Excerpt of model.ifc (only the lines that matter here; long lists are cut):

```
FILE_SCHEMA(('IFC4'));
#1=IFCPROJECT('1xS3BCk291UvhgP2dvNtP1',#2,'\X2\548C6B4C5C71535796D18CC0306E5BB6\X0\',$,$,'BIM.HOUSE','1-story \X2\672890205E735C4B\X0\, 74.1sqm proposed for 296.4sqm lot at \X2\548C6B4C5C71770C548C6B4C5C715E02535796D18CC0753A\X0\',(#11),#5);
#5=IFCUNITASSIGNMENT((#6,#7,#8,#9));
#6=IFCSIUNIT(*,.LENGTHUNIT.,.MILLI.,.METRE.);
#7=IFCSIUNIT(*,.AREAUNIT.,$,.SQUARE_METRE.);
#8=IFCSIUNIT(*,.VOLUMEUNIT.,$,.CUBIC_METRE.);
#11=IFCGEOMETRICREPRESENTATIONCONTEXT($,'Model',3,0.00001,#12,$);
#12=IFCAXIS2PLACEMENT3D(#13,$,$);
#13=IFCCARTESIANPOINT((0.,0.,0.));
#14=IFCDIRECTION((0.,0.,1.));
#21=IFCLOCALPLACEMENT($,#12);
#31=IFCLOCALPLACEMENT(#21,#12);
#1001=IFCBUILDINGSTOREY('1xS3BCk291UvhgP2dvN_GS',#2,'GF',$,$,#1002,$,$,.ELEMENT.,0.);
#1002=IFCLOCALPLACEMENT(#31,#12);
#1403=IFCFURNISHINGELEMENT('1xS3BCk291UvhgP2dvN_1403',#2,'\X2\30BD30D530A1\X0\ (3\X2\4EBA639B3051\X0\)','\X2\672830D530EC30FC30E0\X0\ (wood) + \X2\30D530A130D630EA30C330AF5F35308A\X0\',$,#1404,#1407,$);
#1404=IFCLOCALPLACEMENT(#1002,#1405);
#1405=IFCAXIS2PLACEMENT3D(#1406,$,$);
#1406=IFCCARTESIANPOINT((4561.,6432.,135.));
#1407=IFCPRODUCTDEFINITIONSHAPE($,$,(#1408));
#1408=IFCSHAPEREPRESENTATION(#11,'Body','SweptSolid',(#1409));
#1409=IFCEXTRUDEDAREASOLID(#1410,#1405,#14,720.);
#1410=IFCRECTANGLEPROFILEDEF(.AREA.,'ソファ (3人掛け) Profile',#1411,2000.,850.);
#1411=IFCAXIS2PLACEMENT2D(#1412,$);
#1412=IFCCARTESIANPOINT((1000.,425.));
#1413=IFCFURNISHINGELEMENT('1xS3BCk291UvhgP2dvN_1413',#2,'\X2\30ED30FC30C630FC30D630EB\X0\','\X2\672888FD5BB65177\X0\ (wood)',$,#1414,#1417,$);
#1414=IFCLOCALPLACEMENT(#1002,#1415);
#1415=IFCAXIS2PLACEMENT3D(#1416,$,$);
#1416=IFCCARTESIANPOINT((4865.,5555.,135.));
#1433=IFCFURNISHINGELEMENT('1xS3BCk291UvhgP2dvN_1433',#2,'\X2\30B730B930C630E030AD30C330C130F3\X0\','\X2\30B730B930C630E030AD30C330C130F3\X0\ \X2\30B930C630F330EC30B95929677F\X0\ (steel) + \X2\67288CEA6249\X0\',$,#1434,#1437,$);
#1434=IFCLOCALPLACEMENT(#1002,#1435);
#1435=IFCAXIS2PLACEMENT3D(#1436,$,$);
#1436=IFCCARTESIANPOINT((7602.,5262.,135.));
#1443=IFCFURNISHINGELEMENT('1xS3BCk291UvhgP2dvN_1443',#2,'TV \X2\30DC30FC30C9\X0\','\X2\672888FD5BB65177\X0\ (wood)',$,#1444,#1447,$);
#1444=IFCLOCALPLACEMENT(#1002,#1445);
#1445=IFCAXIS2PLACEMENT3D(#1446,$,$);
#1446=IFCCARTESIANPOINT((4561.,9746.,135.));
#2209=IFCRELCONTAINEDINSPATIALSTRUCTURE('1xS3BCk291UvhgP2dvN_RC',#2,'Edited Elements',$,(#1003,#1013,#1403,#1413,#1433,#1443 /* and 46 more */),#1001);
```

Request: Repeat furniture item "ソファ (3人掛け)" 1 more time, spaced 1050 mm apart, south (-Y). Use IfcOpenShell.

```python
import numpy as np
import ifcopenshell
import ifcopenshell.api.geometry
import ifcopenshell.api.root
import ifcopenshell.util.element
import ifcopenshell.util.placement
import ifcopenshell.util.unit

model = ifcopenshell.open("model.ifc")
unit_scale = ifcopenshell.util.unit.calculate_unit_scale(model)


def reuse_history(source, copy):
    """copy_class also copies each property set's owner history, people and application; keep the originals."""
    for rel in copy.IsDefinedBy:
        if rel.is_a("IfcRelDefinesByProperties") and (history := rel.RelatingPropertyDefinition.OwnerHistory):
            rel.RelatingPropertyDefinition.OwnerHistory = source.OwnerHistory
            ifcopenshell.util.element.remove_deep2(model, history)


source = model.by_guid("1xS3BCk291UvhgP2dvN_1403")
base = ifcopenshell.util.placement.get_local_placement(source.ObjectPlacement)
step = np.array([0.0, -1.0, 0.0]) * 1.05 / unit_scale

for i in range(1, 2):
    copy = ifcopenshell.api.root.copy_class(model, product=source)
    copy.Representation = ifcopenshell.util.element.copy_deep(
        model, source.Representation, exclude=["IfcGeometricRepresentationContext", "IfcRepresentationMap"]
    )
    reuse_history(source, copy)
    matrix = base.copy()
    matrix[:3, 3] += i * step
    print("added at", matrix[:3, 3].round(3) + 0.0)
    ifcopenshell.api.geometry.edit_object_placement(model, product=copy, matrix=matrix, is_si=False)

model.write("model_updated.ifc")
```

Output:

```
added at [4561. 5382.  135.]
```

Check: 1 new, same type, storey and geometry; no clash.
